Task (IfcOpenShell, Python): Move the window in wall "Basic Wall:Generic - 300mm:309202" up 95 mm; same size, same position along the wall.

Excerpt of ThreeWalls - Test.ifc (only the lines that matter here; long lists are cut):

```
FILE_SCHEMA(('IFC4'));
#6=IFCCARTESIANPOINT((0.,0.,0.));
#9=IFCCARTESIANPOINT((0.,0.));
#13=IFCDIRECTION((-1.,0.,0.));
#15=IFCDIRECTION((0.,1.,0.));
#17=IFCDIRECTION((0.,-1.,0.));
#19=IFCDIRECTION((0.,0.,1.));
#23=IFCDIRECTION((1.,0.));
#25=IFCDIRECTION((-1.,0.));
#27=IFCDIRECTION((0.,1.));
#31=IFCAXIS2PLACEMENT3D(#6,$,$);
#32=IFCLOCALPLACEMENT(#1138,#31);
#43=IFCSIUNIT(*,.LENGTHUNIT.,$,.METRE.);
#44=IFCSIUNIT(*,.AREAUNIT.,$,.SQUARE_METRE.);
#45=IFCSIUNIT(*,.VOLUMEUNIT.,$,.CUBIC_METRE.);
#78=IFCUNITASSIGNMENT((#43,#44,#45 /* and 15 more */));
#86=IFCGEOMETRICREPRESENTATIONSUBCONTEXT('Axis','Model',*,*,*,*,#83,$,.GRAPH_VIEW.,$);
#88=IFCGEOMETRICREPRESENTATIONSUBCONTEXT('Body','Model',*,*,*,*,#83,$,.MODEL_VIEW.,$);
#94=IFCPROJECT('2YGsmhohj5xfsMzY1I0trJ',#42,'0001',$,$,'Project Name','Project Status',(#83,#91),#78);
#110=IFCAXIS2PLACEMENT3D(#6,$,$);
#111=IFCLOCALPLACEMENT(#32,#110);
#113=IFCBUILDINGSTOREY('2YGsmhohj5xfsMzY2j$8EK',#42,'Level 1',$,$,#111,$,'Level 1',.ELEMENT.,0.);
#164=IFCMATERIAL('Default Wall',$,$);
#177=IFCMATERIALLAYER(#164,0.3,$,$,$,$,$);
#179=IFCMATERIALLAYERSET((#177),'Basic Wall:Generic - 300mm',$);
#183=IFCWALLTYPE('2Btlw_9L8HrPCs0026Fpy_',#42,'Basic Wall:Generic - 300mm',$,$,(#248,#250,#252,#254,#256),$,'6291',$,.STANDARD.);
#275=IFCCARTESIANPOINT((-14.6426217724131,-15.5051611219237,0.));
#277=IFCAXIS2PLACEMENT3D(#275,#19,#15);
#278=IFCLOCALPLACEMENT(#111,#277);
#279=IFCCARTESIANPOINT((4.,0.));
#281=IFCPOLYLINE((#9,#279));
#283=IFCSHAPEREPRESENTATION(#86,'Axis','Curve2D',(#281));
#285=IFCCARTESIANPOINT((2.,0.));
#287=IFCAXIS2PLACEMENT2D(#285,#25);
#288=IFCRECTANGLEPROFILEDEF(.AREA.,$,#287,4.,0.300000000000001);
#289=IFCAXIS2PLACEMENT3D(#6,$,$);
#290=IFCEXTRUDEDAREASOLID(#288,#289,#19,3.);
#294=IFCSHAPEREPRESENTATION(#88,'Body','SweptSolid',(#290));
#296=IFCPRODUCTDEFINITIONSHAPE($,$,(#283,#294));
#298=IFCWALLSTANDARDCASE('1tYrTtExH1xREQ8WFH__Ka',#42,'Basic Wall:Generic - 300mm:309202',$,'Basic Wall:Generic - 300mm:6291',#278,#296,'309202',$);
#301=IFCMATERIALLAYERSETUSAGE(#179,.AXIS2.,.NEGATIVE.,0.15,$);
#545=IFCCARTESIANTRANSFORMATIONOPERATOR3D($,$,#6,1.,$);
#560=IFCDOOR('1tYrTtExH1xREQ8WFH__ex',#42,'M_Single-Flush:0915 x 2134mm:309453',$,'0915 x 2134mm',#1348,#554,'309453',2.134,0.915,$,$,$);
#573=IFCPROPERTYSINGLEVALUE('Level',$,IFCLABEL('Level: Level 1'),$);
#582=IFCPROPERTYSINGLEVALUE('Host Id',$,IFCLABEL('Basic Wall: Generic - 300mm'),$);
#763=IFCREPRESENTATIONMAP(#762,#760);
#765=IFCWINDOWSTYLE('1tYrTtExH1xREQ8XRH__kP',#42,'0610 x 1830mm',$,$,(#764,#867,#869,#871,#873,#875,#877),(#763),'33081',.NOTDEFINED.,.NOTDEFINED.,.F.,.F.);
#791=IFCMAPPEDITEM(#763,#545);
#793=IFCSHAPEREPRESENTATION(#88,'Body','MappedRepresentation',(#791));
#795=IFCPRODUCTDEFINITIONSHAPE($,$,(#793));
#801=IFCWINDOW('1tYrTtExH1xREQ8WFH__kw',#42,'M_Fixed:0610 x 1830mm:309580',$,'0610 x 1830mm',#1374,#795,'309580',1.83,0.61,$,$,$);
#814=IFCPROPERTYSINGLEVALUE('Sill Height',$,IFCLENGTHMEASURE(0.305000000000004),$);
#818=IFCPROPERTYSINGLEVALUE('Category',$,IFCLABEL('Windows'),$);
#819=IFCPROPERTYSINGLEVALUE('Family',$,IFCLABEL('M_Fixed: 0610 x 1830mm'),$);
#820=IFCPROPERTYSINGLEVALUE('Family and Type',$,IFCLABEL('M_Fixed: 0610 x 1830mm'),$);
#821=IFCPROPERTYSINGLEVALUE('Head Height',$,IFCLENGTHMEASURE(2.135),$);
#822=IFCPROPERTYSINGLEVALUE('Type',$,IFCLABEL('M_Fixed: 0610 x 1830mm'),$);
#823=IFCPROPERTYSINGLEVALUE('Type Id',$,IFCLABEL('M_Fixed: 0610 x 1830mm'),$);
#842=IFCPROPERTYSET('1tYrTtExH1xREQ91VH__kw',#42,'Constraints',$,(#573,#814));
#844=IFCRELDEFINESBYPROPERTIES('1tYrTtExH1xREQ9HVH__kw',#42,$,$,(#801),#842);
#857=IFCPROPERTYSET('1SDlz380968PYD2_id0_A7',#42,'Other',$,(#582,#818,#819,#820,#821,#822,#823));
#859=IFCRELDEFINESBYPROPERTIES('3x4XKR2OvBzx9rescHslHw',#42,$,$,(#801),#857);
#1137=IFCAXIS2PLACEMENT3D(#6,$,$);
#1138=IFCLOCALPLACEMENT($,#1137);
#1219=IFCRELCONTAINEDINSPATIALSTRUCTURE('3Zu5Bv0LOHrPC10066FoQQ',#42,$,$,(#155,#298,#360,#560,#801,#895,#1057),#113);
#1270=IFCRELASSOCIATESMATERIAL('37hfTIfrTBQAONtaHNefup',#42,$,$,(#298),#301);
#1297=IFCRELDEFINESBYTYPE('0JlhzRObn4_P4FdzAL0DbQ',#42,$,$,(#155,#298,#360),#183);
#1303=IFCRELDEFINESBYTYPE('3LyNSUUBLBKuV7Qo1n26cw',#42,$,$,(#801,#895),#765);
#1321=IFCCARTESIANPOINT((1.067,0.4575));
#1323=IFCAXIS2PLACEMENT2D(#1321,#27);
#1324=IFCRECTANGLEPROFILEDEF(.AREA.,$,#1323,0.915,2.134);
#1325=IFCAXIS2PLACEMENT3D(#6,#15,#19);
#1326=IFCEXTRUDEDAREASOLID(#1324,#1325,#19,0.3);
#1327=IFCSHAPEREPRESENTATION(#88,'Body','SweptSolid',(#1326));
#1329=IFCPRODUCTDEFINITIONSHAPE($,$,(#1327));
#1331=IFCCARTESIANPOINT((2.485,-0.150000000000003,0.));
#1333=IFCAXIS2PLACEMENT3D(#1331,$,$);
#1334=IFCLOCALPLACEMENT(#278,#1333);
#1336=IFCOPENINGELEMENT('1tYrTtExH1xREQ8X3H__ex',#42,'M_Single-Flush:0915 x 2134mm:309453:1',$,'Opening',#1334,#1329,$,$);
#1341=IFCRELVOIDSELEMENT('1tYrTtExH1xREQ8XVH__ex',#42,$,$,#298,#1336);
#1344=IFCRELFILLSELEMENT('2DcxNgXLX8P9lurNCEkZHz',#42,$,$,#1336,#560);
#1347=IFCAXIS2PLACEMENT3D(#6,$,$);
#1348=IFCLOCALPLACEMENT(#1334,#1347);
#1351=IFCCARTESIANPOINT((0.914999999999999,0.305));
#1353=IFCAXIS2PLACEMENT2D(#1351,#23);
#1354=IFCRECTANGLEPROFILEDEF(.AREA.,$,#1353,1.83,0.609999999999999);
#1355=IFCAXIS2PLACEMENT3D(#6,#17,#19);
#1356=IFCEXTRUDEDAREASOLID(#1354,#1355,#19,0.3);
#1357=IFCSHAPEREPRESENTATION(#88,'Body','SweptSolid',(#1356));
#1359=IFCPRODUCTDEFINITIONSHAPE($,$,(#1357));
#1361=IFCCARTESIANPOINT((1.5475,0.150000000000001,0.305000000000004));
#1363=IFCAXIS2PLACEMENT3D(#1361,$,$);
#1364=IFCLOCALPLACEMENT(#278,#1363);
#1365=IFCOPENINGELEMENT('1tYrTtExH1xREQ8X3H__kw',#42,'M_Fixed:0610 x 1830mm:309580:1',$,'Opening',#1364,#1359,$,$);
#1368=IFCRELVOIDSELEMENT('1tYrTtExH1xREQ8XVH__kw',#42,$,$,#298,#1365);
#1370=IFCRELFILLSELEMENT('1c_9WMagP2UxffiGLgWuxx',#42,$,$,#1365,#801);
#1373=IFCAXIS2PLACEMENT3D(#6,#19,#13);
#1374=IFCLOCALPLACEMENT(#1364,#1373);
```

```python
import numpy as np
import ifcopenshell
import ifcopenshell.api.geometry
import ifcopenshell.api.pset
import ifcopenshell.util.element
import ifcopenshell.util.placement
import ifcopenshell.util.unit

model = ifcopenshell.open("ThreeWalls - Test.ifc")
unit_scale = ifcopenshell.util.unit.calculate_unit_scale(model)

window = model.by_guid("1tYrTtExH1xREQ8WFH__kw")
opening = window.FillsVoids[0].RelatingOpeningElement
dz = 0.095 / unit_scale

shift = np.array([0.0, 0.0, dz])
# The window is placed relative to its opening, so it follows when the opening moves.
matrix = ifcopenshell.util.placement.get_local_placement(opening.ObjectPlacement)
matrix[:3, 3] += shift
ifcopenshell.api.geometry.edit_object_placement(
    model, product=opening, matrix=matrix, is_si=False, should_transform_children=True
)

# Keep the stored heights in step.
pset = model.by_id(ifcopenshell.util.element.get_pset(window, "Constraints", should_inherit=False)["id"])
ifcopenshell.api.pset.edit_pset(model, pset=pset, properties={
    "Sill Height": model.create_entity("IfcLengthMeasure", ifcopenshell.util.element.get_pset(window, "Constraints", "Sill Height") + dz),
})
pset = model.by_id(ifcopenshell.util.element.get_pset(window, "Other", should_inherit=False)["id"])
ifcopenshell.api.pset.edit_pset(model, pset=pset, properties={
    "Head Height": model.create_entity("IfcLengthMeasure", ifcopenshell.util.element.get_pset(window, "Other", "Head Height") + dz),
})

print(f"moved by {dz * unit_scale:+.3f} m")

model.write("ThreeWalls - Test_edited.ifc")
```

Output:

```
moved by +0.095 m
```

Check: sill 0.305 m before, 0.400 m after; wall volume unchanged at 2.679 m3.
